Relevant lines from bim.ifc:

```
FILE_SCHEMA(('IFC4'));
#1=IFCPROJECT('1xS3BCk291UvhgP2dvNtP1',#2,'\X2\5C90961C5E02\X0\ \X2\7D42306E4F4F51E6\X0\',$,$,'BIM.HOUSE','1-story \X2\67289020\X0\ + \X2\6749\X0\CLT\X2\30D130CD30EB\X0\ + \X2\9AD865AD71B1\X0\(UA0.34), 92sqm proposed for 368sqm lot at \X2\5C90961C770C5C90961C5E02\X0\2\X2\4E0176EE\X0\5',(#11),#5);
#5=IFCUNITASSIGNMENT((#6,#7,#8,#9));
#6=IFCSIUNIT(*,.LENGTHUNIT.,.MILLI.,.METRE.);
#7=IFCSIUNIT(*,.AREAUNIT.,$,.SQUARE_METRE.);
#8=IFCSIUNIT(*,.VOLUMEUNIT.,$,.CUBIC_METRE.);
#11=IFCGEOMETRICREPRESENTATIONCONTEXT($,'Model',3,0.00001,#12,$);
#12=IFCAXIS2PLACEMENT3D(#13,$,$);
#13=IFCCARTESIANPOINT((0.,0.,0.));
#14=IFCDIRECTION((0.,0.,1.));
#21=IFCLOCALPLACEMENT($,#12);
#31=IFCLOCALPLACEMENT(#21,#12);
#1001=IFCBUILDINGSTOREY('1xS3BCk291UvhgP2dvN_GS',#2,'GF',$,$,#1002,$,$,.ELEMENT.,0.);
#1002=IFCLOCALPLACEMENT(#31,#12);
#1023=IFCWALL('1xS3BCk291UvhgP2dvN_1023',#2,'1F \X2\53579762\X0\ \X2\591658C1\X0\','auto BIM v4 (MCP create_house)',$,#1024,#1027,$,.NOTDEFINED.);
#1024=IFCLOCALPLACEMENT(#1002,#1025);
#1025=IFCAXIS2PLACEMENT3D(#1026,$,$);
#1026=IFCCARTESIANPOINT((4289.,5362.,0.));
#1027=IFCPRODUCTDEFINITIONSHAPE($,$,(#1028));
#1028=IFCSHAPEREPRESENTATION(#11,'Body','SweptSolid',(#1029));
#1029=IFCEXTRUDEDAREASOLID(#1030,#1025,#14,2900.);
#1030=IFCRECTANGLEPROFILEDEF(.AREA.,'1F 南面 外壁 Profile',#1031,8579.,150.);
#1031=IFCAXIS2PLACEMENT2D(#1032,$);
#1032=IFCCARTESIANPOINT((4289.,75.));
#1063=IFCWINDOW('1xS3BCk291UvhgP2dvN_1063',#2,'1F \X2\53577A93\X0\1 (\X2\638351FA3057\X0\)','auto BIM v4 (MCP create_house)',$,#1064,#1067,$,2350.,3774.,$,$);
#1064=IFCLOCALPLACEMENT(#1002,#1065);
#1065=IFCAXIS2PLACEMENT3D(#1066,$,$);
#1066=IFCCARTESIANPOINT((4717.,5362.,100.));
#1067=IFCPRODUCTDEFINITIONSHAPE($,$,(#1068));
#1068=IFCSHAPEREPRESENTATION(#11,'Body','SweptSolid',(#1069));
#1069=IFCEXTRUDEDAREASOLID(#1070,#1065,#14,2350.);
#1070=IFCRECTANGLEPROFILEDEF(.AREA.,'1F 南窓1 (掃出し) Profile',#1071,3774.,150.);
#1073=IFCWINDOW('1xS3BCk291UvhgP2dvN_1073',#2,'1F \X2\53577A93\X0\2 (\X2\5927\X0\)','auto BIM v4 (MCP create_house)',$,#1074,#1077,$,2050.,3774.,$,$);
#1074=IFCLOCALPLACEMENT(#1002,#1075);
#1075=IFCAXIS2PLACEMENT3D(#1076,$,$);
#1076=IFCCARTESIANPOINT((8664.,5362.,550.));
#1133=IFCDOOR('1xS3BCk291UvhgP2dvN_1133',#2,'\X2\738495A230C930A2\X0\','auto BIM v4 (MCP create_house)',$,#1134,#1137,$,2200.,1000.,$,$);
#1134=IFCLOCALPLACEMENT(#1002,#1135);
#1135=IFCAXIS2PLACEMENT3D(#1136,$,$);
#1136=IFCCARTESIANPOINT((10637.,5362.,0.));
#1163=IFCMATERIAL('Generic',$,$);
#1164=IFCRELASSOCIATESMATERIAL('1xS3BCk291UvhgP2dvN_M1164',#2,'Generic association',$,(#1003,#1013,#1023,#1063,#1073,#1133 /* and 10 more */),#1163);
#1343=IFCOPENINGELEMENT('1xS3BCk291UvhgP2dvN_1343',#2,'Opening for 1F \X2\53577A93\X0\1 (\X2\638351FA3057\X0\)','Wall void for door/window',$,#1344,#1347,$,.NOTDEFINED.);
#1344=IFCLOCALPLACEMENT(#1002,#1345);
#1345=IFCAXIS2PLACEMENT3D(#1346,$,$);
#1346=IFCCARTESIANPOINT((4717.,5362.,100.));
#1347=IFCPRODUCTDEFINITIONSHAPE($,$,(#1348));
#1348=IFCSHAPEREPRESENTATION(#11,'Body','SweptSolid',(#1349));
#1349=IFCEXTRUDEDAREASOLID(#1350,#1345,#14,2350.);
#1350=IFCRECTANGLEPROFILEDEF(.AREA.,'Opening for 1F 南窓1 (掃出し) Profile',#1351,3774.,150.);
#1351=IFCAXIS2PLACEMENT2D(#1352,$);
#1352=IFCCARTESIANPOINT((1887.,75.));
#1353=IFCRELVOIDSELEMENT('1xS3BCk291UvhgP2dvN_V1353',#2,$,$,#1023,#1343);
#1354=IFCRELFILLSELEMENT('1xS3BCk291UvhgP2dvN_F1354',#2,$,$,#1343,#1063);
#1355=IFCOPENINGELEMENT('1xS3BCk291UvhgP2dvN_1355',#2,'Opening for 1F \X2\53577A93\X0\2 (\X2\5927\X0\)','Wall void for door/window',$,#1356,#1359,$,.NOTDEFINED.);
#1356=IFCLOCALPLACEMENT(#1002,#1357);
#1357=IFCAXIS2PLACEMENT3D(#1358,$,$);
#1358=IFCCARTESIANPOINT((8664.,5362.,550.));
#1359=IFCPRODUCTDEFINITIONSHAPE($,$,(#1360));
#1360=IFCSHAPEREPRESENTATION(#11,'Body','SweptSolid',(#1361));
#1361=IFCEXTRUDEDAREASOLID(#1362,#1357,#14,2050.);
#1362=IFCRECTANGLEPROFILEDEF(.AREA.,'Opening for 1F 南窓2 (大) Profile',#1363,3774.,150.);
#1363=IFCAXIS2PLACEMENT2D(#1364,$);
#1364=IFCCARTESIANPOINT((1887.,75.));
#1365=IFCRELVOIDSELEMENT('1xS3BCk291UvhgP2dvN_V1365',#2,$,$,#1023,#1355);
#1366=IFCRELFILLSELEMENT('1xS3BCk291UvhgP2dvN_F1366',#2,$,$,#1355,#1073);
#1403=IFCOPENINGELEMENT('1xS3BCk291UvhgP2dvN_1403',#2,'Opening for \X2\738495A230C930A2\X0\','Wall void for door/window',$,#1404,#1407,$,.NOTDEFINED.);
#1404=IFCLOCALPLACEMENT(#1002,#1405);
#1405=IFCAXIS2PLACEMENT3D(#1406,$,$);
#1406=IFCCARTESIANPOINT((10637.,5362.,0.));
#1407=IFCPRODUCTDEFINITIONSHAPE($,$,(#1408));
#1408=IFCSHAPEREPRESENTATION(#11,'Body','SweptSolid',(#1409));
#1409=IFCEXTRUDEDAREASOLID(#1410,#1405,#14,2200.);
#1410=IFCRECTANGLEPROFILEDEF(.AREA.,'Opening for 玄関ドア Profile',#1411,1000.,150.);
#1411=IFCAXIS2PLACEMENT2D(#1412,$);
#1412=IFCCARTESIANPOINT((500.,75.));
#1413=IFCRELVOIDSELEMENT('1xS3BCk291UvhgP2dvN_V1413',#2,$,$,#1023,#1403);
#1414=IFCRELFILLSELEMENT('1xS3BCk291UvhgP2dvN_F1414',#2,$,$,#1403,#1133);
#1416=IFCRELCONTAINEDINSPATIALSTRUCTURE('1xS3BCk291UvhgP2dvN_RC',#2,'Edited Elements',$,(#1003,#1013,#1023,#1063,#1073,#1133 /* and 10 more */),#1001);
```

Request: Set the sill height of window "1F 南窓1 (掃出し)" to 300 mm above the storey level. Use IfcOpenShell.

```python
import numpy as np
import ifcopenshell
import ifcopenshell.api.geometry
import ifcopenshell.geom
import ifcopenshell.util.element
import ifcopenshell.util.placement
import ifcopenshell.util.shape
import ifcopenshell.util.unit

model = ifcopenshell.open("bim.ifc")
unit_scale = ifcopenshell.util.unit.calculate_unit_scale(model)

window = model.by_id(1063)
opening = window.FillsVoids[0].RelatingOpeningElement
storey = ifcopenshell.util.element.get_container(window, ifc_class="IfcBuildingStorey")
level = ifcopenshell.util.placement.get_local_placement(storey.ObjectPlacement)[2, 3]

# The opening's origin need not be at the sill, so measure its lowest point.
shape = ifcopenshell.geom.create_shape(ifcopenshell.geom.settings(), opening)
bottom = ifcopenshell.util.shape.get_shape_bottom_elevation(shape, shape.geometry) / unit_scale
dz = level + 300.0 - bottom

shift = np.array([0.0, 0.0, dz])
# The window is not placed relative to its opening, so move both.
for product in (opening, window):
    matrix = ifcopenshell.util.placement.get_local_placement(product.ObjectPlacement)
    matrix[:3, 3] += shift
    ifcopenshell.api.geometry.edit_object_placement(model, product=product, matrix=matrix, is_si=False)

print(f"moved by {dz * unit_scale:+.3f} m")

model.write("bim_edited.ifc")
```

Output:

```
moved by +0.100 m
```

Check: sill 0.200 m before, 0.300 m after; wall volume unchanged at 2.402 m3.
